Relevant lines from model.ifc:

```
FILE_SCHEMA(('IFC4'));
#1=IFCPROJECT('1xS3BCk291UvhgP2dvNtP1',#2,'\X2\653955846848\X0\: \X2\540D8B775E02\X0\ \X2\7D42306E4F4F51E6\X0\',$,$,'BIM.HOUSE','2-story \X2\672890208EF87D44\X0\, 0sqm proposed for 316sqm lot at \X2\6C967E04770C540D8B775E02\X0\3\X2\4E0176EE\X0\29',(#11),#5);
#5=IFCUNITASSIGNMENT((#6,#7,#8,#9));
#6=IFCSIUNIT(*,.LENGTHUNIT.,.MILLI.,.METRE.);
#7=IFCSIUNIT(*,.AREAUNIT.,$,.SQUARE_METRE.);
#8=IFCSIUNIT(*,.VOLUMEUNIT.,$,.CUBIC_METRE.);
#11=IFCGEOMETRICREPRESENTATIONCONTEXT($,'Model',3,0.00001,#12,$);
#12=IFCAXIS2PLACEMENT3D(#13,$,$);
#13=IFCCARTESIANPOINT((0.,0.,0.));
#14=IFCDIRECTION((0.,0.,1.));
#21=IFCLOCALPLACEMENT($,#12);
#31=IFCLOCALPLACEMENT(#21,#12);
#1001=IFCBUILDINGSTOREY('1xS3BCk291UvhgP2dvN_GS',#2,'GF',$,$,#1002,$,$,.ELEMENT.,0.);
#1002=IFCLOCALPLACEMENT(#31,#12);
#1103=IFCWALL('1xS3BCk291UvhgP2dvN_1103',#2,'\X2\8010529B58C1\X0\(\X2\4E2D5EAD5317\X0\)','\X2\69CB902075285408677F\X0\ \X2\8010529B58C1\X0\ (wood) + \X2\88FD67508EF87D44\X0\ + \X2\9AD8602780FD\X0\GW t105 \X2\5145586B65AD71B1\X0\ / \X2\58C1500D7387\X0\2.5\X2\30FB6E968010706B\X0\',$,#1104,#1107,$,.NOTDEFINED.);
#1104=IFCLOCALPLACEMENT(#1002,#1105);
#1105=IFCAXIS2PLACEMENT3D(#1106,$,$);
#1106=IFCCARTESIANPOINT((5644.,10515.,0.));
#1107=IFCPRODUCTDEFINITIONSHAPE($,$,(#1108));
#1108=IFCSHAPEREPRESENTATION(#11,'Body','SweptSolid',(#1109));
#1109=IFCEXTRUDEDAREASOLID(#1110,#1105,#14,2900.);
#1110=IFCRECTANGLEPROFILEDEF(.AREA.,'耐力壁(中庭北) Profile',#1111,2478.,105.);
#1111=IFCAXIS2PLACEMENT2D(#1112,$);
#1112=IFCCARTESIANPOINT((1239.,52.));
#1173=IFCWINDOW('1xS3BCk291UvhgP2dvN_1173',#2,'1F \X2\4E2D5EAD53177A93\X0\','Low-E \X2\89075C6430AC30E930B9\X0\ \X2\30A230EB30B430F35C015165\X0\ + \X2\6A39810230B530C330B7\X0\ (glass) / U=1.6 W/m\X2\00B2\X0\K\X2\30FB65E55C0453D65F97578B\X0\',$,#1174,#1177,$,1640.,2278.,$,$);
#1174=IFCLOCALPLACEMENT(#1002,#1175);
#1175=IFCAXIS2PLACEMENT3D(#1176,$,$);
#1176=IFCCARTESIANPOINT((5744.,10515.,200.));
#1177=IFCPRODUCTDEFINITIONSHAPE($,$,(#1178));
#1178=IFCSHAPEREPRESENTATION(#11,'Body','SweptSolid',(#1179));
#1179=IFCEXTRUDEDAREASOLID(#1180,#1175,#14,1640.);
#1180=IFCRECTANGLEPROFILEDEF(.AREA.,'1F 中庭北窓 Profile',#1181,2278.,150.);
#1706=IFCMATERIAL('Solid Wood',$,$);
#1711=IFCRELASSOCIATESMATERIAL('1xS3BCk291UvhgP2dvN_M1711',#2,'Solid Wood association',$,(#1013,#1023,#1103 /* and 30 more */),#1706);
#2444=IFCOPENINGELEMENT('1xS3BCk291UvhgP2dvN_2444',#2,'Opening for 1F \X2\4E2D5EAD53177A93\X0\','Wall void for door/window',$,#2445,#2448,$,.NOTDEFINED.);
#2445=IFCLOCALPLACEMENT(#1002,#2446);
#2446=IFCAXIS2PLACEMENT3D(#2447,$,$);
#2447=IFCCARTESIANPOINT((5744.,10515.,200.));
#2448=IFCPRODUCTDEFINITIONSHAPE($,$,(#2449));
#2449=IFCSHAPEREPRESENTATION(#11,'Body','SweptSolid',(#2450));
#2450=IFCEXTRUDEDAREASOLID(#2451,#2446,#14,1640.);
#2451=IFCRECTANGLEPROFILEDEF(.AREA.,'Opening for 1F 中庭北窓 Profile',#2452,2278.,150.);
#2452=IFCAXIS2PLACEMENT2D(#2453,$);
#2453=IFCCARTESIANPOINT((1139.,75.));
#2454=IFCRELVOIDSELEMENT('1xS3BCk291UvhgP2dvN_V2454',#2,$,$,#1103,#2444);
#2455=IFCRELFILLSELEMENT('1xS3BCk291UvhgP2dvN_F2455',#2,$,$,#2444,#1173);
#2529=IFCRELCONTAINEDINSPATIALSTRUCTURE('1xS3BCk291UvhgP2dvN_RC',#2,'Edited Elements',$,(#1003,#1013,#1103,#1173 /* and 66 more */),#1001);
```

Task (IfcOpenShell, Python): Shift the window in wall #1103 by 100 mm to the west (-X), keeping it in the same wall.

```python
import ifcopenshell
import ifcopenshell.api.geometry
import ifcopenshell.util.placement
import ifcopenshell.util.unit

model = ifcopenshell.open("model.ifc")
unit_scale = ifcopenshell.util.unit.calculate_unit_scale(model)

window = model.by_guid("1xS3BCk291UvhgP2dvN_1173")
opening = window.FillsVoids[0].RelatingOpeningElement
wall = opening.VoidsElements[0].RelatingBuildingElement

wall_matrix = ifcopenshell.util.placement.get_local_placement(wall.ObjectPlacement)
shift = wall_matrix[:3, 0] * -0.1 / unit_scale
before = ifcopenshell.util.placement.get_local_placement(window.ObjectPlacement)[:3, 3].copy()

# The window is not placed relative to its opening, so move both.
for product in (opening, window):
    matrix = ifcopenshell.util.placement.get_local_placement(product.ObjectPlacement)
    matrix[:3, 3] += shift
    ifcopenshell.api.geometry.edit_object_placement(model, product=product, matrix=matrix, is_si=False)

after = ifcopenshell.util.placement.get_local_placement(window.ObjectPlacement)[:3, 3]
print("window moved by", (after - before).round(3) + 0.0)

model.write("model-out.ifc")
```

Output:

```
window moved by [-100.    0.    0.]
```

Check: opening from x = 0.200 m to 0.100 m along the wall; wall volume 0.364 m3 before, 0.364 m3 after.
